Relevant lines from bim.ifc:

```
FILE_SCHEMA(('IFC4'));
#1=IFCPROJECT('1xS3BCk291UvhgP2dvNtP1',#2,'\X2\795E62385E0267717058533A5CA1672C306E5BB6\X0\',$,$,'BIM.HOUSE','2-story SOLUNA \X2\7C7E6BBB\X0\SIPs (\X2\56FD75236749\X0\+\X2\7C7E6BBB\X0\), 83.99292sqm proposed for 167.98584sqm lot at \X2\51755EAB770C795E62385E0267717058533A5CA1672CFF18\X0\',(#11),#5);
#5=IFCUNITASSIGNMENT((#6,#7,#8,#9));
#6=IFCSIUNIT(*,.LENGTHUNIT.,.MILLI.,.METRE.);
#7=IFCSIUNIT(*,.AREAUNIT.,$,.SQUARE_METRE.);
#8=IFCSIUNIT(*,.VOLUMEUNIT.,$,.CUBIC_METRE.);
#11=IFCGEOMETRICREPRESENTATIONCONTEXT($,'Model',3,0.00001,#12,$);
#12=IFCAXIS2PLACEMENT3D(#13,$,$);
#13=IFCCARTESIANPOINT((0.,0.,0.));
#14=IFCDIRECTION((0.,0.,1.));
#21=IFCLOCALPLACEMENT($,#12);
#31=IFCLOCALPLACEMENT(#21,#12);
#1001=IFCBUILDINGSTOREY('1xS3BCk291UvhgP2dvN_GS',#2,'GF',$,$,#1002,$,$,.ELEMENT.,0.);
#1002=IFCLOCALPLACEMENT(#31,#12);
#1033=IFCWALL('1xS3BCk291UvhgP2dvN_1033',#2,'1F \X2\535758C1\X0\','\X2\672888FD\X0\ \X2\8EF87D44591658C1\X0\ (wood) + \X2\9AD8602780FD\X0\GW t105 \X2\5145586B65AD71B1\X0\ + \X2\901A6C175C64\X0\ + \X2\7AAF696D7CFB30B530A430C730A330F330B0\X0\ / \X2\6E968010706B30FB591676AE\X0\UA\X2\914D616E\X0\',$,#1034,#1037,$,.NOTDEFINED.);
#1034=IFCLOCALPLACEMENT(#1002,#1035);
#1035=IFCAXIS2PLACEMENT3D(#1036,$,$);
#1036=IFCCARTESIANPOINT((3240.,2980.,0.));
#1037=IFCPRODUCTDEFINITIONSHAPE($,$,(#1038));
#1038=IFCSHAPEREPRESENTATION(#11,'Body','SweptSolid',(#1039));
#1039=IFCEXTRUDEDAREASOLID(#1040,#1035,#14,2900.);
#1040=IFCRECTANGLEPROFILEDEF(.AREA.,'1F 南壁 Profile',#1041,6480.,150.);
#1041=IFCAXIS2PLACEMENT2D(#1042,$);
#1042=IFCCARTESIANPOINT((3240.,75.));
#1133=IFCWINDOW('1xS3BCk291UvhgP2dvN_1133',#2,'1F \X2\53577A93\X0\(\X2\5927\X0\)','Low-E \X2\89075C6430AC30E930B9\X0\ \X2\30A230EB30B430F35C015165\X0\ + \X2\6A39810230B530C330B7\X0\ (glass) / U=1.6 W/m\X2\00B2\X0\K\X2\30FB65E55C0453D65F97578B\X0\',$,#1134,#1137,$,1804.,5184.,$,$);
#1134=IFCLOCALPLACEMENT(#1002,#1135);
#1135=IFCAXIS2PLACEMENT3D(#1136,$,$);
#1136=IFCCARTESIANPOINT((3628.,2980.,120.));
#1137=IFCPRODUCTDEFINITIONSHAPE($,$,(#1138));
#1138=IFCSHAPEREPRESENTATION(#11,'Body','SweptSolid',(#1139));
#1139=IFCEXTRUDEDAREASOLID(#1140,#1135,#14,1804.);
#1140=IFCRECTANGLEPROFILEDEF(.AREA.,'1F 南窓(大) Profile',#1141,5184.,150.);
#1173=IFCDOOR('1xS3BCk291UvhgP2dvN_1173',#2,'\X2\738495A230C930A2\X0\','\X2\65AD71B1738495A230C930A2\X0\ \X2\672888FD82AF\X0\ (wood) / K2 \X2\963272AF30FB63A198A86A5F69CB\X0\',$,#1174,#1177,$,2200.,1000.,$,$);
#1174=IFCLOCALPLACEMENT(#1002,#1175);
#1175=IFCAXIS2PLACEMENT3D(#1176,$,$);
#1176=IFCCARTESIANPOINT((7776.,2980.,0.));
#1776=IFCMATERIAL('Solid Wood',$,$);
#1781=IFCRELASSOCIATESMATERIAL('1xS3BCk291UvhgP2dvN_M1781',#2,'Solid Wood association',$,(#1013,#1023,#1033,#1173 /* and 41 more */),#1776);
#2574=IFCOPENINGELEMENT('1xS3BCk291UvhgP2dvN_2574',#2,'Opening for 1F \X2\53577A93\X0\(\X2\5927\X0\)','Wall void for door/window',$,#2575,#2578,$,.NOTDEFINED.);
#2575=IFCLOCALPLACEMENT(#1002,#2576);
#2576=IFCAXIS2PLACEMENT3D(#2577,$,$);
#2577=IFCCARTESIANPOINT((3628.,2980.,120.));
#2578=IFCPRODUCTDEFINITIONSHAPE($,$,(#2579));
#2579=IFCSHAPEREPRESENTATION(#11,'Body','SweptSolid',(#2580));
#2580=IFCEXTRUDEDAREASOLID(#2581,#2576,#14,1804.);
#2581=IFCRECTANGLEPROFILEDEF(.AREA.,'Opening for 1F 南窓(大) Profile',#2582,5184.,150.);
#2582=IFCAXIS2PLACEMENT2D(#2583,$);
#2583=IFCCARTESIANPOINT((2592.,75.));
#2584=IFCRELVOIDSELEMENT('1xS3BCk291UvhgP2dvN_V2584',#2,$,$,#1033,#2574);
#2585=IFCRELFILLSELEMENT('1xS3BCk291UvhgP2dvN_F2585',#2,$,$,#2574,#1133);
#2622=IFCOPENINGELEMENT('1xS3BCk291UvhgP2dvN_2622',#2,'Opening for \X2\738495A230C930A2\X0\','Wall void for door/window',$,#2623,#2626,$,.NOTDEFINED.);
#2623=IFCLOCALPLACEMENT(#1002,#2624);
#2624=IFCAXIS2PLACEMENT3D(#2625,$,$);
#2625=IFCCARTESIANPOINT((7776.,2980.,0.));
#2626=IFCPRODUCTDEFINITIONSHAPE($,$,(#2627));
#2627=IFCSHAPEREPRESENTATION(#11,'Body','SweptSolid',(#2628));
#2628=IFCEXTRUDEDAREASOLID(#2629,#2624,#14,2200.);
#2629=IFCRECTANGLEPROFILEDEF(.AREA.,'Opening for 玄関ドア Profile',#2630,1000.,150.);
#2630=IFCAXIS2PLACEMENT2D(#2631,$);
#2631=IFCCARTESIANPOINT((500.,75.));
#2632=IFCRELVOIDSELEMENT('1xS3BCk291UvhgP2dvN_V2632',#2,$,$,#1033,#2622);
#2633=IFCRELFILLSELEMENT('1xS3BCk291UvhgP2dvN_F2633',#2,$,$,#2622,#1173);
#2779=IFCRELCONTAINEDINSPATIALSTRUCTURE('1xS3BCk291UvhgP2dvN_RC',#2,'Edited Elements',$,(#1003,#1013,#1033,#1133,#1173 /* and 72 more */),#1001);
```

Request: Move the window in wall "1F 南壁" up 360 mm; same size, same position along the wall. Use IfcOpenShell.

```python
import numpy as np
import ifcopenshell
import ifcopenshell.api.geometry
import ifcopenshell.util.placement
import ifcopenshell.util.unit

model = ifcopenshell.open("bim.ifc")
unit_scale = ifcopenshell.util.unit.calculate_unit_scale(model)

window = model.by_id(1133)
opening = window.FillsVoids[0].RelatingOpeningElement
dz = 360.0

shift = np.array([0.0, 0.0, dz])
# The window is not placed relative to its opening, so move both.
for product in (opening, window):
    matrix = ifcopenshell.util.placement.get_local_placement(product.ObjectPlacement)
    matrix[:3, 3] += shift
    ifcopenshell.api.geometry.edit_object_placement(model, product=product, matrix=matrix, is_si=False)

print(f"moved by {dz * unit_scale:+.3f} m")

model.write("bim-out.ifc")
```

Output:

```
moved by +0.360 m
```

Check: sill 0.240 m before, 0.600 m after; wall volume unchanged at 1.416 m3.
